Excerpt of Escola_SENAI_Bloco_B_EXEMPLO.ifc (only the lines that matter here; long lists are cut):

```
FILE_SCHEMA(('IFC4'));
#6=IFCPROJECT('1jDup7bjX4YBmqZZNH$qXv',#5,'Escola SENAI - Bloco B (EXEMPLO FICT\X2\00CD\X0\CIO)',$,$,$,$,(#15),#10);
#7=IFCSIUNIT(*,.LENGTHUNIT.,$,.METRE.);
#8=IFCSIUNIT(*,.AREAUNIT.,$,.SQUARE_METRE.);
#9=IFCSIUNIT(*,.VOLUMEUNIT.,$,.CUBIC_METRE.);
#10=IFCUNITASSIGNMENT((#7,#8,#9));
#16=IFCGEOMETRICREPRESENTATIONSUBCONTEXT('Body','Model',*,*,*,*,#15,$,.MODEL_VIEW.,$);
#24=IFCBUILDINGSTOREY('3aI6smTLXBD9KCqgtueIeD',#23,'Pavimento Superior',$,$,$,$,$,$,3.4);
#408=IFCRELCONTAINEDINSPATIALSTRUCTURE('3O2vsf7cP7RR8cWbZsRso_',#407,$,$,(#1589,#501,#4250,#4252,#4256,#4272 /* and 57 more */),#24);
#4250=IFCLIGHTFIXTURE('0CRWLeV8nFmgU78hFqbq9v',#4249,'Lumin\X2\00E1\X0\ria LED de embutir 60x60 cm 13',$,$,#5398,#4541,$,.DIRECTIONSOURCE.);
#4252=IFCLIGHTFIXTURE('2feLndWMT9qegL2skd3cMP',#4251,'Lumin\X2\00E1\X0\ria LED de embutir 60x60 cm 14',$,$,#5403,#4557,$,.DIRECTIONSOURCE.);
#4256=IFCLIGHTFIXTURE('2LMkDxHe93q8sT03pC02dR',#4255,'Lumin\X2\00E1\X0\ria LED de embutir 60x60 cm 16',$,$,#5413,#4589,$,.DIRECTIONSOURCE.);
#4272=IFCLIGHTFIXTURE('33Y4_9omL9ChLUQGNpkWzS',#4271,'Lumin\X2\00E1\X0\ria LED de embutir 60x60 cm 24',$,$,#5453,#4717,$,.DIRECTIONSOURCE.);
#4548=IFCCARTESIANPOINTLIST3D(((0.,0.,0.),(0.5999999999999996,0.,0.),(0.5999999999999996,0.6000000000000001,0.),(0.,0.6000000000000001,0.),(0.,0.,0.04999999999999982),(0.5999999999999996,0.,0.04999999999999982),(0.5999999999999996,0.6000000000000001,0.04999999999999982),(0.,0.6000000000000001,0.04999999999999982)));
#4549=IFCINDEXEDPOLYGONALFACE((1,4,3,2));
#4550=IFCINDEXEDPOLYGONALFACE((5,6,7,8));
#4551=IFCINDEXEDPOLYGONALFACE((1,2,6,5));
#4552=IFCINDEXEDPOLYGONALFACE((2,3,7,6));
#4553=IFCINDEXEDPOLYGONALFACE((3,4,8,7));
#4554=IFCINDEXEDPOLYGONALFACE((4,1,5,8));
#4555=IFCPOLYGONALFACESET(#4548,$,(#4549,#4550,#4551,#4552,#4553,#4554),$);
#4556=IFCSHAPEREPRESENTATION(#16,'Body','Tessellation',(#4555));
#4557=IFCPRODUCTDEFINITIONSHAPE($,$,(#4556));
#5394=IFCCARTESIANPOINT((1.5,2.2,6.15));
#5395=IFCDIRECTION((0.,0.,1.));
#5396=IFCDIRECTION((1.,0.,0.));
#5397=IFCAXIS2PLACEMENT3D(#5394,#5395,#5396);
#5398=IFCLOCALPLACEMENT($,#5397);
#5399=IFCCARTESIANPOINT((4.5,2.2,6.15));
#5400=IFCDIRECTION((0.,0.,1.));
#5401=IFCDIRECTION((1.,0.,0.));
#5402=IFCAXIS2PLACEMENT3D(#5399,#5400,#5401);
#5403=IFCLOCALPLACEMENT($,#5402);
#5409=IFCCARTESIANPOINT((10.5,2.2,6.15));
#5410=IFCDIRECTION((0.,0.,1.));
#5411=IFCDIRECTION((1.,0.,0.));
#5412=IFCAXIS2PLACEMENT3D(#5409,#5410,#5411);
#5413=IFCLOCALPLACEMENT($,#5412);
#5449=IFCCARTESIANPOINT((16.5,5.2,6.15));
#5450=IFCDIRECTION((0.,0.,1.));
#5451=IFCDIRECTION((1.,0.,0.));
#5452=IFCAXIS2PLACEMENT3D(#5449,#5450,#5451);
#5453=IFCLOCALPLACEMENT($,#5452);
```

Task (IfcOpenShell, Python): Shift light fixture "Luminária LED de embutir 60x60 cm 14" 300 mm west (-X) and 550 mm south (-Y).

```python
import ifcopenshell
import ifcopenshell.api.geometry
import ifcopenshell.util.placement

model = ifcopenshell.open("Escola_SENAI_Bloco_B_EXEMPLO.ifc")

item = model.by_guid("2feLndWMT9qegL2skd3cMP")
matrix = ifcopenshell.util.placement.get_local_placement(item.ObjectPlacement)
matrix[0, 3] -= 0.3
matrix[1, 3] -= 0.55
ifcopenshell.api.geometry.edit_object_placement(model, product=item, matrix=matrix, is_si=False)

print(ifcopenshell.util.placement.get_local_placement(item.ObjectPlacement).round(3) + 0.0)

model.write("Escola_SENAI_Bloco_B_EXEMPLO_edited.ifc")
```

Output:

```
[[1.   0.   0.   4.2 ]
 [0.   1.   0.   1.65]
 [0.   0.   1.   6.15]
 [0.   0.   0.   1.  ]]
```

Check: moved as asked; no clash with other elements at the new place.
